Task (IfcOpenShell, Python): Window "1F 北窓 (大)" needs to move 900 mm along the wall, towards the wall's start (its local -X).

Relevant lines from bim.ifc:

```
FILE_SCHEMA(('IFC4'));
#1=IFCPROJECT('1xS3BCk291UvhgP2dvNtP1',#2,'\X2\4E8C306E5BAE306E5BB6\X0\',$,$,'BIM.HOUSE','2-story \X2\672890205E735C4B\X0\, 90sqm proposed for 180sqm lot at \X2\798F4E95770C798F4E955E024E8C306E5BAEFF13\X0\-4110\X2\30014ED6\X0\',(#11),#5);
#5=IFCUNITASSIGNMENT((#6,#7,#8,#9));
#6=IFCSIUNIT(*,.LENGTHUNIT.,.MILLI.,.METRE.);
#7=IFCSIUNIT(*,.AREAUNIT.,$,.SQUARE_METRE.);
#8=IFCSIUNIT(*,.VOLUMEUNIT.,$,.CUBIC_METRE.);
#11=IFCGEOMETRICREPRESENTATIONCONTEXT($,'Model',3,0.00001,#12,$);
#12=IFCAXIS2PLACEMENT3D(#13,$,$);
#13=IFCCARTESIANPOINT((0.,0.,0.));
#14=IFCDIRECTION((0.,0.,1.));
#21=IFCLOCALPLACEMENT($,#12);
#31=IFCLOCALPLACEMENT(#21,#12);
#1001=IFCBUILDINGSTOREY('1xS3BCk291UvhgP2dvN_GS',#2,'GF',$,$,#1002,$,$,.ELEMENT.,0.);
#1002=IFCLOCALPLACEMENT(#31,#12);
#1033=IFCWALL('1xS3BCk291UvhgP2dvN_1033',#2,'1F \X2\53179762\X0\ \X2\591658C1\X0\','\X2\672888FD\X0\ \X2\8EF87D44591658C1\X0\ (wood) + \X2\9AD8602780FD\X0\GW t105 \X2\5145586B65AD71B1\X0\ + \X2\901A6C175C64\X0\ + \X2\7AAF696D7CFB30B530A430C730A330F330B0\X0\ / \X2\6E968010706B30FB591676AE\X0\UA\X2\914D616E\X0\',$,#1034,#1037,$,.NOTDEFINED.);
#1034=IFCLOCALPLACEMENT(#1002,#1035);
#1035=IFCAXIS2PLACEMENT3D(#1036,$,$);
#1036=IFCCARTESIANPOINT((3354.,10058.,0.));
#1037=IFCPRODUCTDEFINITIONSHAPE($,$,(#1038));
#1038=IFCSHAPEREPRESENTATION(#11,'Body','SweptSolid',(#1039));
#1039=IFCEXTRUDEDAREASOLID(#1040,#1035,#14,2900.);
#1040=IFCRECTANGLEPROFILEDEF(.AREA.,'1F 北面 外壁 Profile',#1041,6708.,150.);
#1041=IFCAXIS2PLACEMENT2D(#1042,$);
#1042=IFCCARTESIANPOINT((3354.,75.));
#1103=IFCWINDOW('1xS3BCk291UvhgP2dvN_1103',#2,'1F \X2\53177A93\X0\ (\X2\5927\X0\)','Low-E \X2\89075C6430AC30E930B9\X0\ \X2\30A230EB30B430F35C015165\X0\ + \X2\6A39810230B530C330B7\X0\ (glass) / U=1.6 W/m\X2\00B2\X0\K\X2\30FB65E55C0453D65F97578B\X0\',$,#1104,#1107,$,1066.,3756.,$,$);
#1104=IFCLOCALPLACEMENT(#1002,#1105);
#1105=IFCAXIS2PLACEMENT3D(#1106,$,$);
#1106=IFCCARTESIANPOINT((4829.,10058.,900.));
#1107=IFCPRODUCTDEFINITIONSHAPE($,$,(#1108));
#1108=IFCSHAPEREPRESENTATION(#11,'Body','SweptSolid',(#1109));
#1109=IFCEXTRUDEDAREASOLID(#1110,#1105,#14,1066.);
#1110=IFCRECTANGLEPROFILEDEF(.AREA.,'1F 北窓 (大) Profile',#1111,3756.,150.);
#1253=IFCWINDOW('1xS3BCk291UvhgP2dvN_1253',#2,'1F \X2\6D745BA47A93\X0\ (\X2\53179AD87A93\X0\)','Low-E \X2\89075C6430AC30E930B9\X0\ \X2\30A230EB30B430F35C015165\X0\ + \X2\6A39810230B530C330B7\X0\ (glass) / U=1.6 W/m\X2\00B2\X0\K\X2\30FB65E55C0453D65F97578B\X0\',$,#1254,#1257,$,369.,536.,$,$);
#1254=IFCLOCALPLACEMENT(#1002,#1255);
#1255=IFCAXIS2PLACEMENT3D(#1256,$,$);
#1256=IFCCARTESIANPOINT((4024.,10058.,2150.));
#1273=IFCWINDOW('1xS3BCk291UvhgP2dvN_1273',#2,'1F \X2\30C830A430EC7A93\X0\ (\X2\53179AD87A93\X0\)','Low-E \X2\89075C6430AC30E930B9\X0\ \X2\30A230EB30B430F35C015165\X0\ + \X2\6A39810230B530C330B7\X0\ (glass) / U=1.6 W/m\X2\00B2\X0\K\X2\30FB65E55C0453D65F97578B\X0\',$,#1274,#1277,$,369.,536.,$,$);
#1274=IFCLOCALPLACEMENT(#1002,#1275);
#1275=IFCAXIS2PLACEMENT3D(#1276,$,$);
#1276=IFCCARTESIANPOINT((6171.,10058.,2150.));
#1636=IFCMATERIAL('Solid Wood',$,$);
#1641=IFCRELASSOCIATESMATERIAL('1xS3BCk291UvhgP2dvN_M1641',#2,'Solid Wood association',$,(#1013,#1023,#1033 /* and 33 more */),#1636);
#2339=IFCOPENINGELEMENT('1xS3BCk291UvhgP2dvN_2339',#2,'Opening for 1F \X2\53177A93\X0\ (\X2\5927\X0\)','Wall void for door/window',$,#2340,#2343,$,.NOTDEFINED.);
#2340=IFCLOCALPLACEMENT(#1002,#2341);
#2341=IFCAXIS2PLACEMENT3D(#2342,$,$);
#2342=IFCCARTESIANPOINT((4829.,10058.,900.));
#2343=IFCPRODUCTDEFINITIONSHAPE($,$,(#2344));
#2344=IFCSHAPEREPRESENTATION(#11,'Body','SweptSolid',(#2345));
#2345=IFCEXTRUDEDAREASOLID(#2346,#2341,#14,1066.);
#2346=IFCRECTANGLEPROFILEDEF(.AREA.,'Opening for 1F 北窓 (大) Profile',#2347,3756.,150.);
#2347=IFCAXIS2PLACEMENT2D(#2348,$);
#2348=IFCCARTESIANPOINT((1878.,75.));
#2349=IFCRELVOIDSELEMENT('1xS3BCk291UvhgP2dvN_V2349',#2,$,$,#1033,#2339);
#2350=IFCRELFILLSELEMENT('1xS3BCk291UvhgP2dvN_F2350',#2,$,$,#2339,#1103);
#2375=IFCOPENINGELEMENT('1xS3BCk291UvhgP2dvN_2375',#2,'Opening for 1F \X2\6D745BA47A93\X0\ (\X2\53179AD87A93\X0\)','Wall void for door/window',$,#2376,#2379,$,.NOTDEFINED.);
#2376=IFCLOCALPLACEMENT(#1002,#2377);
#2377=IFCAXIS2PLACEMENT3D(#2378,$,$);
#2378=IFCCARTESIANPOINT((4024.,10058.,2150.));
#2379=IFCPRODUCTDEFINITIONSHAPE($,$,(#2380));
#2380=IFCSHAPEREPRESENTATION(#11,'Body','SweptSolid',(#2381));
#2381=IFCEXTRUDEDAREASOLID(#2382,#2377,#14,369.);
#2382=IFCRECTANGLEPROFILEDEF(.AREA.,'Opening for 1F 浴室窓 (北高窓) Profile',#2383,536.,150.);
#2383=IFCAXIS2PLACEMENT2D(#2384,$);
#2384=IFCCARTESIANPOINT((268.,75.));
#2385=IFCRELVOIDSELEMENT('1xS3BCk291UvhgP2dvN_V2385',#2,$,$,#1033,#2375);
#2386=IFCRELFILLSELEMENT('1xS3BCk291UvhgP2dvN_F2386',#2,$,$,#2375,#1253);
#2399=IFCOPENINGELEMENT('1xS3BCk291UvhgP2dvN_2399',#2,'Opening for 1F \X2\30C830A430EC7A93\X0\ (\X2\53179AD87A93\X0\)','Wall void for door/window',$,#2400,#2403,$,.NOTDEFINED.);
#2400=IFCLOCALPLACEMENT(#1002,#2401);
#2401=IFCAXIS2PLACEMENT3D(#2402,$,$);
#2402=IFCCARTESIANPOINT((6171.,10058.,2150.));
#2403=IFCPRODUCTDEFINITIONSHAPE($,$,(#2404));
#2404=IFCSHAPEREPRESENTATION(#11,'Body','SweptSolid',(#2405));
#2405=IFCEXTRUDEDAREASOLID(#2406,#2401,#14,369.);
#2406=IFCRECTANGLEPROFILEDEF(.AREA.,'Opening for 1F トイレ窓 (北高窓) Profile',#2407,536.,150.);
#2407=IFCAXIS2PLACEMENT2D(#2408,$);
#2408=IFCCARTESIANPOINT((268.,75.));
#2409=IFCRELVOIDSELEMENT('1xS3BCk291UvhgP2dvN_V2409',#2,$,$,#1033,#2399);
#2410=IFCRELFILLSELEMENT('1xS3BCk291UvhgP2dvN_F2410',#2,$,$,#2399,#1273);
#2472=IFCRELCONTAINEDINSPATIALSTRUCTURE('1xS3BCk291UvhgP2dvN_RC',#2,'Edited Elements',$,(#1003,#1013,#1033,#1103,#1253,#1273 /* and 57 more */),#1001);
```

```python
import ifcopenshell
import ifcopenshell.api.geometry
import ifcopenshell.util.placement
import ifcopenshell.util.unit

model = ifcopenshell.open("bim.ifc")
unit_scale = ifcopenshell.util.unit.calculate_unit_scale(model)

window = model.by_id(1103)
opening = window.FillsVoids[0].RelatingOpeningElement
wall = opening.VoidsElements[0].RelatingBuildingElement

wall_matrix = ifcopenshell.util.placement.get_local_placement(wall.ObjectPlacement)
shift = wall_matrix[:3, 0] * -0.9 / unit_scale
before = ifcopenshell.util.placement.get_local_placement(window.ObjectPlacement)[:3, 3].copy()

# The window is not placed relative to its opening, so move both.
for product in (opening, window):
    matrix = ifcopenshell.util.placement.get_local_placement(product.ObjectPlacement)
    matrix[:3, 3] += shift
    ifcopenshell.api.geometry.edit_object_placement(model, product=product, matrix=matrix, is_si=False)

after = ifcopenshell.util.placement.get_local_placement(window.ObjectPlacement)[:3, 3]
print("window moved by", (after - before).round(3) + 0.0)

model.write("bim_rev.ifc")
```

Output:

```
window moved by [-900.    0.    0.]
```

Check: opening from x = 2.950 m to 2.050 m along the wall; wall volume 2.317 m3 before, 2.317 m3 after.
